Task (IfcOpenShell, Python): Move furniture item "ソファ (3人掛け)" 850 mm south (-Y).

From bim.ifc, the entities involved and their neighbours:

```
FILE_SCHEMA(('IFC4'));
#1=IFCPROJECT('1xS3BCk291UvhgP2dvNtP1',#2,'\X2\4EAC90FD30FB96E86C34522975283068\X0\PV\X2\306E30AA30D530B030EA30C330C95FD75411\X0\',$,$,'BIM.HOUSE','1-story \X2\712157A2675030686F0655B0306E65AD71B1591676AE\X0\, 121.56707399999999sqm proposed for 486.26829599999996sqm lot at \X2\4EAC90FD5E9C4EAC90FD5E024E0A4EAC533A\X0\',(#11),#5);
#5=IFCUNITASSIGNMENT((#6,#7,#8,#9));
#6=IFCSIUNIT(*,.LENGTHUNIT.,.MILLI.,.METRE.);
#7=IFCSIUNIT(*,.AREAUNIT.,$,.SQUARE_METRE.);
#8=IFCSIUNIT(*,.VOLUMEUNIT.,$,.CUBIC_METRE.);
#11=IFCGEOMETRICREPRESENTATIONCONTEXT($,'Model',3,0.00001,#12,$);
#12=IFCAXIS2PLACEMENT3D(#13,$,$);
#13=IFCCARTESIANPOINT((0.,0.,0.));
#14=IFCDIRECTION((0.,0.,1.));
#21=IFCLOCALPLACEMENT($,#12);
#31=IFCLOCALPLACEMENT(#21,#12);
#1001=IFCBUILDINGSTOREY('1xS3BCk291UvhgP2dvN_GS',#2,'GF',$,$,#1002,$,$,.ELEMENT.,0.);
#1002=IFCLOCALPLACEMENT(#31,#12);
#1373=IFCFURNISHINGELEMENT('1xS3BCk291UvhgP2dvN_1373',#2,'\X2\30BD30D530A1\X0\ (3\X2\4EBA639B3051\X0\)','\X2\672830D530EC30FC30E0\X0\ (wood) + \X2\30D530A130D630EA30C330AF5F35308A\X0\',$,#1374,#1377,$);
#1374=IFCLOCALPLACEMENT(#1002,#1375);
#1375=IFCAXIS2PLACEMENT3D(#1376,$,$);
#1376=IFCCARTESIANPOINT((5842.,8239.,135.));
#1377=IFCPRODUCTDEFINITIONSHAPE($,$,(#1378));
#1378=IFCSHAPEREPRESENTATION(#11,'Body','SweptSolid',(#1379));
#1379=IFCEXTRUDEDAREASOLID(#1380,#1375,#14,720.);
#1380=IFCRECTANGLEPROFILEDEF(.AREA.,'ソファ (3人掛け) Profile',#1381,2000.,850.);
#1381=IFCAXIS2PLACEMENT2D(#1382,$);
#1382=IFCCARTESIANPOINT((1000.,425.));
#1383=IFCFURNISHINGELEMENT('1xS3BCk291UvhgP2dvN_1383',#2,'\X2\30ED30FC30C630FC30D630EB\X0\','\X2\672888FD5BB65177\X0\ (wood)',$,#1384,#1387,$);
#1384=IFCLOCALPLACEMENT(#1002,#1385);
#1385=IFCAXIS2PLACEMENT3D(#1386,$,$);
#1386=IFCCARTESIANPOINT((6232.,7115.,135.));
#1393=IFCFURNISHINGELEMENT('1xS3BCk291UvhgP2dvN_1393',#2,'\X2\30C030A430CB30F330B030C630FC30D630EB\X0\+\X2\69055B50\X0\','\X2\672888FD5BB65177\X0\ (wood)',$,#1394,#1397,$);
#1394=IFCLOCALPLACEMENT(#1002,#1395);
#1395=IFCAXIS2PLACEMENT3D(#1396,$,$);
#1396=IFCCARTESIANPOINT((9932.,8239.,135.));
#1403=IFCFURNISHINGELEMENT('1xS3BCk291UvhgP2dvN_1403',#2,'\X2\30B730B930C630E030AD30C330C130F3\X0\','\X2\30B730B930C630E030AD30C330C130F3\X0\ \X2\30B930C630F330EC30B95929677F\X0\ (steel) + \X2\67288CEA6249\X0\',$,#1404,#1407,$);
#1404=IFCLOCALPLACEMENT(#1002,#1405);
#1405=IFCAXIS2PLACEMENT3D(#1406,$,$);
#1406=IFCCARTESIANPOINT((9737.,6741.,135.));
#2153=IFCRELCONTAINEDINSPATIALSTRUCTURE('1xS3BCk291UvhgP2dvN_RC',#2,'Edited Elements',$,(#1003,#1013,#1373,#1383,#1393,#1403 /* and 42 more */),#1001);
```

```python
import ifcopenshell
import ifcopenshell.api.geometry
import ifcopenshell.util.placement

model = ifcopenshell.open("bim.ifc")

item = model.by_guid("1xS3BCk291UvhgP2dvN_1373")
matrix = ifcopenshell.util.placement.get_local_placement(item.ObjectPlacement)
matrix[1, 3] -= 850.0
ifcopenshell.api.geometry.edit_object_placement(model, product=item, matrix=matrix, is_si=False)

print(ifcopenshell.util.placement.get_local_placement(item.ObjectPlacement).round(3) + 0.0)

model.write("bim_updated.ifc")
```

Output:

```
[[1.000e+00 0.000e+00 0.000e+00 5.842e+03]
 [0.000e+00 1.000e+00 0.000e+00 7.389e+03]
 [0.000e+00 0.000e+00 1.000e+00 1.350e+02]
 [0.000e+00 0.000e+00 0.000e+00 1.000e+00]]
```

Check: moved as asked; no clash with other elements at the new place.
